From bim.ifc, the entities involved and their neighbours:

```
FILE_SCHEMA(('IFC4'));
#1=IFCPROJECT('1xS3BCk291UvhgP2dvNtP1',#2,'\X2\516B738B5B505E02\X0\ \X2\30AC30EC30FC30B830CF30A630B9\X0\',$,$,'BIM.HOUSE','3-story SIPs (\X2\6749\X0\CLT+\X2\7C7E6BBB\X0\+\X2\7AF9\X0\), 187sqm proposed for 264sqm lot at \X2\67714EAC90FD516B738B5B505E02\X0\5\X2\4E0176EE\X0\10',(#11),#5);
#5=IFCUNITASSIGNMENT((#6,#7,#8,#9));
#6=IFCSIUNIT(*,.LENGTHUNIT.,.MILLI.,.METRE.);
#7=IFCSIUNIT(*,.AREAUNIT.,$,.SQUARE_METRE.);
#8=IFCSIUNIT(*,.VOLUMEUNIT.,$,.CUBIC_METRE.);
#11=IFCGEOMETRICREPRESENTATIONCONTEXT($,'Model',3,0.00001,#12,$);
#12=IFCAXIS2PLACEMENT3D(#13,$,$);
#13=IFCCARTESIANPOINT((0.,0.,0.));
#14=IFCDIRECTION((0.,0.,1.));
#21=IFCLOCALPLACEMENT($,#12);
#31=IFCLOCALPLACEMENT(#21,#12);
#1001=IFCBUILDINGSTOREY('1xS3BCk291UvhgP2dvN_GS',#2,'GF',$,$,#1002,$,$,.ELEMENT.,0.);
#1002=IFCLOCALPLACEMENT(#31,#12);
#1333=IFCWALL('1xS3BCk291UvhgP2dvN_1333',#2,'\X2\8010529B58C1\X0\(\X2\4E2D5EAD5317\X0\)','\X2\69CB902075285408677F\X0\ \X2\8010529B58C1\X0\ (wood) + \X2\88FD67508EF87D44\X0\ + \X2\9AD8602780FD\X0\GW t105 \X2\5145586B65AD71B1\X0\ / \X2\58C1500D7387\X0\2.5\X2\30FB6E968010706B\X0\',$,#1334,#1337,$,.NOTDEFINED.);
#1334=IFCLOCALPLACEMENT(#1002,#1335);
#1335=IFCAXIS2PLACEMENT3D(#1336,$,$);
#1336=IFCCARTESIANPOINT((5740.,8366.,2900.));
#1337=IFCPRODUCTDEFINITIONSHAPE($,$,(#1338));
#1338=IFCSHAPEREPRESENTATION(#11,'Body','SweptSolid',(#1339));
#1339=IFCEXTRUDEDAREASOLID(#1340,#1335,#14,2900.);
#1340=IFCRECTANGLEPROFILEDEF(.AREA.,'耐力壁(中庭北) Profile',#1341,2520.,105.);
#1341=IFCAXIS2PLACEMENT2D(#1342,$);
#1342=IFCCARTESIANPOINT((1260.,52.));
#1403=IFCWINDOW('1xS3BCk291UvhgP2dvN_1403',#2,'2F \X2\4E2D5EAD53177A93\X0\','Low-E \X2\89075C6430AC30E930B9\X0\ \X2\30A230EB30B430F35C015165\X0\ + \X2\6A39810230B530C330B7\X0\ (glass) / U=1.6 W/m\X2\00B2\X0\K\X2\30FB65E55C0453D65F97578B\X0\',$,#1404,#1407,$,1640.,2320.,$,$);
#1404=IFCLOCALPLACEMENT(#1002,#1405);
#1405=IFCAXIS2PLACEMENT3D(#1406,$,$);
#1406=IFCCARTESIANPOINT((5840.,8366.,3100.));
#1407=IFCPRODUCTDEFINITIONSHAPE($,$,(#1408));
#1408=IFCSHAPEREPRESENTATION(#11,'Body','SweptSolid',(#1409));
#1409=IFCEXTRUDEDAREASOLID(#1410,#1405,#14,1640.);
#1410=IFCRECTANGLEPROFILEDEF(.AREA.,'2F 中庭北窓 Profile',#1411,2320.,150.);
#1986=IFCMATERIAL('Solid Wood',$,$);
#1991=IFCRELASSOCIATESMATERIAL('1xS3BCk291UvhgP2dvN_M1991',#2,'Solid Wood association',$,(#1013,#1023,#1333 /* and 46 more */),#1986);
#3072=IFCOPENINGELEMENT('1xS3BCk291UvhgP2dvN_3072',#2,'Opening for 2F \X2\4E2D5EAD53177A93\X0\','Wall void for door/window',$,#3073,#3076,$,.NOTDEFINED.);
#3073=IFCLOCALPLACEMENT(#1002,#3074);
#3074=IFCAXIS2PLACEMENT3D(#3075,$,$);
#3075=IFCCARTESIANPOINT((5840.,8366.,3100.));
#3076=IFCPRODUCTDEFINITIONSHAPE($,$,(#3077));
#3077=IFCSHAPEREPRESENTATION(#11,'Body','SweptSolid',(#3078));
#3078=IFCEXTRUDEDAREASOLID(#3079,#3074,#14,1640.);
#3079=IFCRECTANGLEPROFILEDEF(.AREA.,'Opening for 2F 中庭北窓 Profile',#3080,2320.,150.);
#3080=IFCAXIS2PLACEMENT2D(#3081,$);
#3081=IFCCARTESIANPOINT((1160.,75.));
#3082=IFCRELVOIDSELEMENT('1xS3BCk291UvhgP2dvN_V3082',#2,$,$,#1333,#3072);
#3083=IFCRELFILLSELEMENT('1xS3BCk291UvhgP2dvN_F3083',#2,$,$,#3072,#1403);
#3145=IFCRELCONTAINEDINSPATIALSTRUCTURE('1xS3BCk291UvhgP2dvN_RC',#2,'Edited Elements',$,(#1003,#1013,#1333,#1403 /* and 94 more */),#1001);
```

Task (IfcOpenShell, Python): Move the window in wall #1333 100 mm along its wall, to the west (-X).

```python
import ifcopenshell
import ifcopenshell.api.geometry
import ifcopenshell.util.placement

model = ifcopenshell.open("bim.ifc")

window = model.by_guid("1xS3BCk291UvhgP2dvN_1403")
opening = window.FillsVoids[0].RelatingOpeningElement
wall = opening.VoidsElements[0].RelatingBuildingElement

wall_matrix = ifcopenshell.util.placement.get_local_placement(wall.ObjectPlacement)
shift = wall_matrix[:3, 0] * -100.0
before = ifcopenshell.util.placement.get_local_placement(window.ObjectPlacement)[:3, 3].copy()

# The window is not placed relative to its opening, so move both.
for product in (opening, window):
    matrix = ifcopenshell.util.placement.get_local_placement(product.ObjectPlacement)
    matrix[:3, 3] += shift
    ifcopenshell.api.geometry.edit_object_placement(model, product=product, matrix=matrix, is_si=False)

after = ifcopenshell.util.placement.get_local_placement(window.ObjectPlacement)[:3, 3]
print("window moved by", (after - before).round(3) + 0.0)

model.write("bim_edited.ifc")
```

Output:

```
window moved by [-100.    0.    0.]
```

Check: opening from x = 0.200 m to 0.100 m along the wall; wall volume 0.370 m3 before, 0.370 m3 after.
